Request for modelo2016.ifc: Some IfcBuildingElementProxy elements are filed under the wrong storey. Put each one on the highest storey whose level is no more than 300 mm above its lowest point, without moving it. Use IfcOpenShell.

First a look at what the model holds.

```python
import ifcopenshell
import ifcopenshell.util.element
import ifcopenshell.util.placement

model = ifcopenshell.open("modelo2016.ifc")
print(model.schema)
for storey in model.by_type("IfcBuildingStorey"):
    level = ifcopenshell.util.placement.get_storey_elevation(storey)
    count = sum(e.is_a("IfcBuildingElementProxy") for e in ifcopenshell.util.element.get_contained(storey))
    print(storey.id(), storey.Name, round(level, 3), count, sep=" | ")
```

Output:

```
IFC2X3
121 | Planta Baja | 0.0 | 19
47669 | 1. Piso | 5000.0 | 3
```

```python
import ifcopenshell
import ifcopenshell.api.spatial
import ifcopenshell.geom
import ifcopenshell.util.element
import ifcopenshell.util.placement
import ifcopenshell.util.shape
import ifcopenshell.util.unit

model = ifcopenshell.open("modelo2016.ifc")
unit_scale = ifcopenshell.util.unit.calculate_unit_scale(model)
settings = ifcopenshell.geom.settings()

levels = sorted(
    ((ifcopenshell.util.placement.get_storey_elevation(s) * unit_scale, s) for s in model.by_type("IfcBuildingStorey")),
    key=lambda pair: pair[0],
)

for e in model.by_type("IfcBuildingElementProxy"):
    current = e.ContainedInStructure[0].RelatingStructure if e.ContainedInStructure else None
    if current is None or not current.is_a("IfcBuildingStorey"):
        continue
    shape = ifcopenshell.geom.create_shape(settings, e)
    bottom = ifcopenshell.util.shape.get_shape_bottom_elevation(shape, shape.geometry)
    below = [s for level, s in levels if level <= bottom + 0.3]
    storey = below[-1] if below else levels[0][1]
    if storey != current:
        # assign_container keeps the world position.
        ifcopenshell.api.spatial.assign_container(model, products=[e], relating_structure=storey)
        print(e.id(), current.Name, "->", storey.Name)

model.write("modelo2016_v2.ifc")
```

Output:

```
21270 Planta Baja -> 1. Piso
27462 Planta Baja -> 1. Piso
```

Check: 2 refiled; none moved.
